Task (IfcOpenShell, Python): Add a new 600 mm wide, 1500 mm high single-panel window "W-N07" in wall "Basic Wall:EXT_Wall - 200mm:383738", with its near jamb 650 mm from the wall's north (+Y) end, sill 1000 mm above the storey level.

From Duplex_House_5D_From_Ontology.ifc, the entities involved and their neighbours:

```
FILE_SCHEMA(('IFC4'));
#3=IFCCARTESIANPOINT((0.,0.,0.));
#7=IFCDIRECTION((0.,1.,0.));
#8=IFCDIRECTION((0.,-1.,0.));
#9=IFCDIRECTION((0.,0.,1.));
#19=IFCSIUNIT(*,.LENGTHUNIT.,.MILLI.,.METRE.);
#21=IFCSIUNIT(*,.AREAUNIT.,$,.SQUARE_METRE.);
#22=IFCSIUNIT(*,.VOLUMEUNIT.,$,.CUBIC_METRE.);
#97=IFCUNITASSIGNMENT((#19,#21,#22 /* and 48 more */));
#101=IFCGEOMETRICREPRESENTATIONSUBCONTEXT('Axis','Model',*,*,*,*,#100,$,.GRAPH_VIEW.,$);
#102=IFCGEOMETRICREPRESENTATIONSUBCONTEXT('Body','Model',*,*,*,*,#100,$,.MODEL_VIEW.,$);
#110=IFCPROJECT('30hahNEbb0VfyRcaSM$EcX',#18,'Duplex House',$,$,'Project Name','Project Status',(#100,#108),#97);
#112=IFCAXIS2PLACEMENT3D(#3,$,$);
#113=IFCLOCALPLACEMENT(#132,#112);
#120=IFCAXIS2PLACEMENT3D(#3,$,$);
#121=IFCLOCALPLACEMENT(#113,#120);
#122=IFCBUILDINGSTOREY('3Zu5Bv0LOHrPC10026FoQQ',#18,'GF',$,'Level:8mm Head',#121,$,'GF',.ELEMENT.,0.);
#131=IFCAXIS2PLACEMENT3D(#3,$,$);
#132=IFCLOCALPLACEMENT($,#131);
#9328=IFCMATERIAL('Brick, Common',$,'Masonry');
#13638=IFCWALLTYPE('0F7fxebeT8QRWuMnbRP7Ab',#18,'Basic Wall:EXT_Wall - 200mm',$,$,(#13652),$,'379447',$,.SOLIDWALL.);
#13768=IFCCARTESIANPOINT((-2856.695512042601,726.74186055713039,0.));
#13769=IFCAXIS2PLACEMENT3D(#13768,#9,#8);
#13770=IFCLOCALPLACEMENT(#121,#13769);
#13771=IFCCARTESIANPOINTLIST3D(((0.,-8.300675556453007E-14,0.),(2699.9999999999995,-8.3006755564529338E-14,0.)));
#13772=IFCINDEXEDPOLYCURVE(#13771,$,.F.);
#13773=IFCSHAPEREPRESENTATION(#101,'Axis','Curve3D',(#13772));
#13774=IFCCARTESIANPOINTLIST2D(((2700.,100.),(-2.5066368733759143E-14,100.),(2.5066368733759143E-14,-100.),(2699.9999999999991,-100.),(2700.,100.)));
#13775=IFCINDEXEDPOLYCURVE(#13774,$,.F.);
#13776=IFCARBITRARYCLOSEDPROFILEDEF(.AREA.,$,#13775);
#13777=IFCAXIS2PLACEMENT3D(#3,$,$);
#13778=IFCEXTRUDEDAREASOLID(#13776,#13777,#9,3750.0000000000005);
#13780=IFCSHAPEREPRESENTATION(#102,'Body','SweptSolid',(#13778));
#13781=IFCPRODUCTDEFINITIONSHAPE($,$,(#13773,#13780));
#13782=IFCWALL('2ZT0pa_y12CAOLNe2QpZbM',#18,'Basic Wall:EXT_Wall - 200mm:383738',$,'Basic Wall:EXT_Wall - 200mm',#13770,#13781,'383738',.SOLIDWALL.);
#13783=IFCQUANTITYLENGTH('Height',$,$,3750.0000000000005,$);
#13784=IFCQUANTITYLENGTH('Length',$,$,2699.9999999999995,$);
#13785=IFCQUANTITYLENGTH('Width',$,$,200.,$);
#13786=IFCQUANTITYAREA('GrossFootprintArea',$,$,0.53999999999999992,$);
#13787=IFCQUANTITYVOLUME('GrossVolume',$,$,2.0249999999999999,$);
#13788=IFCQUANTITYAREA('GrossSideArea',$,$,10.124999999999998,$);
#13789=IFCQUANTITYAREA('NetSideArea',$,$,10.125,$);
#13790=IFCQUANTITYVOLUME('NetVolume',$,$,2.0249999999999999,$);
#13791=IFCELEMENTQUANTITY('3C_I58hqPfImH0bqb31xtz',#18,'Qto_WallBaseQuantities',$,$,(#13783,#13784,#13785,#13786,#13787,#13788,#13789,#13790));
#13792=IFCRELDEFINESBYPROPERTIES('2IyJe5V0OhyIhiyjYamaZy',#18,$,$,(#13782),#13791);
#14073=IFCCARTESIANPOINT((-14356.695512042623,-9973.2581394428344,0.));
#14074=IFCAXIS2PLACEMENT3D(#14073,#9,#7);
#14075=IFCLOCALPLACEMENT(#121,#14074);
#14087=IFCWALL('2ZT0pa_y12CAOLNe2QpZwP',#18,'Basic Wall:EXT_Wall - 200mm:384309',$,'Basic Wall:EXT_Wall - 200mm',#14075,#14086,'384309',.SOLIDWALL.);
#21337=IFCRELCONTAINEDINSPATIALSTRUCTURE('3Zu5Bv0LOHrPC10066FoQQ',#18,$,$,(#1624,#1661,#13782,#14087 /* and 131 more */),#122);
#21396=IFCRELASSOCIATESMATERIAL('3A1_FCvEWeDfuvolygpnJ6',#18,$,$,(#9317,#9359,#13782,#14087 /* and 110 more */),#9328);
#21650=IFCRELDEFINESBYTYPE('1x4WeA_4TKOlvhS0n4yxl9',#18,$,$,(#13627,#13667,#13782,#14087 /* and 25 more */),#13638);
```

```python
import numpy as np
import ifcopenshell
import ifcopenshell.api.feature
import ifcopenshell.api.geometry
import ifcopenshell.api.pset
import ifcopenshell.api.root
import ifcopenshell.api.spatial
import ifcopenshell.geom
import ifcopenshell.util.element
import ifcopenshell.util.placement
import ifcopenshell.util.representation
import ifcopenshell.util.shape
import ifcopenshell.util.unit

model = ifcopenshell.open("Duplex_House_5D_From_Ontology.ifc")
unit_scale = ifcopenshell.util.unit.calculate_unit_scale(model)
area_scale = ifcopenshell.util.unit.calculate_unit_scale(model, "AREAUNIT")
volume_scale = ifcopenshell.util.unit.calculate_unit_scale(model, "VOLUMEUNIT")
settings = ifcopenshell.geom.settings()


def volume(element):
    """Net volume in cubic metres, openings subtracted."""
    shape = ifcopenshell.geom.create_shape(settings, element)
    return ifcopenshell.util.shape.get_volume(shape.geometry)


wall = model.by_guid("2ZT0pa_y12CAOLNe2QpZbM")
storey = ifcopenshell.util.element.get_container(wall, ifc_class="IfcBuildingStorey")
context = ifcopenshell.util.representation.get_context(model, "Model", "Body", "MODEL_VIEW")
before = volume(wall)

width, height, from_end, sill = 0.6, 1.5, 0.65, 1  # metres

# The wall runs along its own X axis, and the end named is its -X end.
wall_shape = ifcopenshell.geom.create_shape(settings, wall)
x, y, z = ifcopenshell.util.shape.get_vertices(wall_shape.geometry).T
start = x.min() + from_end
face, thickness = float(y.min()), float(y.max() - y.min())
wall_matrix = ifcopenshell.util.placement.get_local_placement(wall.ObjectPlacement)
level = ifcopenshell.util.placement.get_local_placement(storey.ObjectPlacement)[2, 3]


def in_wall(x, y):
    """Placement at x, y metres in the wall's axes, at sill height."""
    matrix = wall_matrix.copy()
    matrix[:, 3] = wall_matrix @ np.array([x / unit_scale, y / unit_scale, 0.0, 1.0])
    matrix[2, 3] = level + sill / unit_scale
    return matrix


# Opening: a box that overshoots both wall faces by 50 mm.
opening = ifcopenshell.api.root.create_entity(model, ifc_class="IfcOpeningElement", predefined_type="OPENING")
box = ifcopenshell.api.geometry.add_wall_representation(
    model, context=context, length=width, height=height, thickness=thickness + 0.1
)
ifcopenshell.api.geometry.assign_representation(model, product=opening, representation=box)
ifcopenshell.api.geometry.edit_object_placement(model, product=opening, matrix=in_wall(start, face - 0.05), is_si=False)
ifcopenshell.api.feature.add_feature(model, feature=opening, element=wall)

window = ifcopenshell.api.root.create_entity(model, ifc_class="IfcWindow", name="W-N07", predefined_type="WINDOW")
window.OverallWidth, window.OverallHeight = width / unit_scale, height / unit_scale
window.PartitioningType = "SINGLE_PANEL"
body = ifcopenshell.api.geometry.add_window_representation(
    model,
    context=context,
    overall_width=window.OverallWidth,
    overall_height=window.OverallHeight,
    partition_type="SINGLE_PANEL",
)
ifcopenshell.api.geometry.assign_representation(model, product=window, representation=body)
ifcopenshell.api.spatial.assign_container(model, products=[window], relating_structure=storey)
ifcopenshell.api.feature.add_filling(model, opening=opening, element=window)

# Centre the window in the wall's thickness.
ifcopenshell.api.geometry.edit_object_placement(model, product=window, matrix=in_wall(start, face), is_si=False)
window_shape = ifcopenshell.geom.create_shape(settings, window)
depth = ifcopenshell.util.shape.get_vertices(window_shape.geometry)[:, 1]
offset = face + thickness / 2 - (depth.min() + depth.max()) / 2
ifcopenshell.api.geometry.edit_object_placement(model, product=window, matrix=in_wall(start, offset), is_si=False)

after = volume(wall)

# Update the wall's stored quantities.
qto = model.by_id(ifcopenshell.util.element.get_pset(wall, "Qto_WallBaseQuantities", should_inherit=False)["id"])
ifcopenshell.api.pset.edit_qto(model, qto=qto, properties={
    "NetSideArea": after / thickness / area_scale,
    "NetVolume": after / volume_scale,
})

print(f"wall volume {before:.3f} -> {after:.3f} m3")

model.write("Duplex_House_5D_From_Ontology_v2.ifc")
```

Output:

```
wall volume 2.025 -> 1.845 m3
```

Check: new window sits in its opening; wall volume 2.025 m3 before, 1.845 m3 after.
